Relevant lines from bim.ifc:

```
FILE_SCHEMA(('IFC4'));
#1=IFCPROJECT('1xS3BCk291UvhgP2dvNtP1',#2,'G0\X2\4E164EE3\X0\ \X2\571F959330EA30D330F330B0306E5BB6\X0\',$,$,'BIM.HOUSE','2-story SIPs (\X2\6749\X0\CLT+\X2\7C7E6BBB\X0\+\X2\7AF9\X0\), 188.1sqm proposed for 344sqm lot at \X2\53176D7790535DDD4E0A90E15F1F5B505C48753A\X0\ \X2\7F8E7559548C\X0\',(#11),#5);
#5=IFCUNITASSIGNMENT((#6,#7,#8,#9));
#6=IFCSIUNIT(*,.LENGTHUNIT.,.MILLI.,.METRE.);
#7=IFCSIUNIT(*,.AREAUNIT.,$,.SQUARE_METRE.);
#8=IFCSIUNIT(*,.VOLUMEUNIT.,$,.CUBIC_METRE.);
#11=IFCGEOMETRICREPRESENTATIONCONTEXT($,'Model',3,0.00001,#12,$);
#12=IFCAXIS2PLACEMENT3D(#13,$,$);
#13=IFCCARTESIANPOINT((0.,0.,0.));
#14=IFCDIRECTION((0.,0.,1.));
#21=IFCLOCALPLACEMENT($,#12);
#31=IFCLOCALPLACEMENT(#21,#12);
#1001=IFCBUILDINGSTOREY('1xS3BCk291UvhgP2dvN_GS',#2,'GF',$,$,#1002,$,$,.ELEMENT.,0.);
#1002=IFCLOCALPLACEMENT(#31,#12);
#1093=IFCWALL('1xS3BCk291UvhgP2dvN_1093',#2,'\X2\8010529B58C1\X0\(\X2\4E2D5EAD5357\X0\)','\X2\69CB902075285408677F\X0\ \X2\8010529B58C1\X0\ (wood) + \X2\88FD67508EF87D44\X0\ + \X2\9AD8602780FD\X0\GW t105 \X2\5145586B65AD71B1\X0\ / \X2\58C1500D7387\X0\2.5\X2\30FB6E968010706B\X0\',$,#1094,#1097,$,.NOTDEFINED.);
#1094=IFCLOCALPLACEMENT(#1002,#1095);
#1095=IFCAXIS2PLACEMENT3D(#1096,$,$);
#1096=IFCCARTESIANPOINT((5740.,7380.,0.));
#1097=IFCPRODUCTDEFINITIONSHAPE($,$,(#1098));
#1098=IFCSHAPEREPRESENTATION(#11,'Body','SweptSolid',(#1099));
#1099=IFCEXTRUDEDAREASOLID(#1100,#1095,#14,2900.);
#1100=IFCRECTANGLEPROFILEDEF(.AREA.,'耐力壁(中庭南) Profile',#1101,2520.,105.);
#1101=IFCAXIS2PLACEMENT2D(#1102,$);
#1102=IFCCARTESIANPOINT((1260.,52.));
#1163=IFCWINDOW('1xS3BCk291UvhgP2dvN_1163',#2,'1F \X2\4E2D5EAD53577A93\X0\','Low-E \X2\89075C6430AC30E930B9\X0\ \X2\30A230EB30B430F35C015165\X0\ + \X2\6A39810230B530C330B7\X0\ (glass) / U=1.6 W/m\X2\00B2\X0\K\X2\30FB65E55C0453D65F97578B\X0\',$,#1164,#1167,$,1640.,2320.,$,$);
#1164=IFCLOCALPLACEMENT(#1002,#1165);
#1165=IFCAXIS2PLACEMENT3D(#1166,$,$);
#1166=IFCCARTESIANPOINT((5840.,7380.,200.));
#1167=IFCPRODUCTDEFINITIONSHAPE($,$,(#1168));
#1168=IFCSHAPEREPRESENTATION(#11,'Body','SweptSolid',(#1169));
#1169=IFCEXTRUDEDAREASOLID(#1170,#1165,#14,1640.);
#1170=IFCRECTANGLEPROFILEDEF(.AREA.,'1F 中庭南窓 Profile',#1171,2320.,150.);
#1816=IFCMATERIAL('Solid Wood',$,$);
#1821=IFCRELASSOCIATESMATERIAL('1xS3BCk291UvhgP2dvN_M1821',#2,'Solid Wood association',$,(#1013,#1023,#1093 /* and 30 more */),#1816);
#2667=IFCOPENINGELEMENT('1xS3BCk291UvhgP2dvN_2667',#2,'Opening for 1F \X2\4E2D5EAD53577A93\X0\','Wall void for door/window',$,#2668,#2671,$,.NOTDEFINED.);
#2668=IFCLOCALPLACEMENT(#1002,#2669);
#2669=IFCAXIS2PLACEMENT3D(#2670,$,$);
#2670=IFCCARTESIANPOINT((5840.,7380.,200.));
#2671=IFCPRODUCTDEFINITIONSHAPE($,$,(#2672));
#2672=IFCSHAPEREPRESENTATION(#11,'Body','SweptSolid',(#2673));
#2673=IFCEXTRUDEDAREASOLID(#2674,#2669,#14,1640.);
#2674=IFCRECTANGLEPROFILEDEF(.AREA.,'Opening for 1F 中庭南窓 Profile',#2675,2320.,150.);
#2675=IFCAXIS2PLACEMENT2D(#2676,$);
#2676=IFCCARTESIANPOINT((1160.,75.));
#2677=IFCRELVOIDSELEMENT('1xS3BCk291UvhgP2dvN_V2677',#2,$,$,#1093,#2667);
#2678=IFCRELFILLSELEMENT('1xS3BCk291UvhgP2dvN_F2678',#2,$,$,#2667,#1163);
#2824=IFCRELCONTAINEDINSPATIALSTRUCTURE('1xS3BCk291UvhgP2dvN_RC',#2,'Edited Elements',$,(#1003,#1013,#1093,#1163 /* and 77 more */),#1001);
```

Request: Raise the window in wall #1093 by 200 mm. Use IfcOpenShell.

```python
import numpy as np
import ifcopenshell
import ifcopenshell.api.geometry
import ifcopenshell.util.placement
import ifcopenshell.util.unit

model = ifcopenshell.open("bim.ifc")
unit_scale = ifcopenshell.util.unit.calculate_unit_scale(model)

window = model.by_guid("1xS3BCk291UvhgP2dvN_1163")
opening = window.FillsVoids[0].RelatingOpeningElement
dz = 200.0

shift = np.array([0.0, 0.0, dz])
# The window is not placed relative to its opening, so move both.
for product in (opening, window):
    matrix = ifcopenshell.util.placement.get_local_placement(product.ObjectPlacement)
    matrix[:3, 3] += shift
    ifcopenshell.api.geometry.edit_object_placement(model, product=product, matrix=matrix, is_si=False)

print(f"moved by {dz * unit_scale:+.3f} m")

model.write("bim_v2.ifc")
```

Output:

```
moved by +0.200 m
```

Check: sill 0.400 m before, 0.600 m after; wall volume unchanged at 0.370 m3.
